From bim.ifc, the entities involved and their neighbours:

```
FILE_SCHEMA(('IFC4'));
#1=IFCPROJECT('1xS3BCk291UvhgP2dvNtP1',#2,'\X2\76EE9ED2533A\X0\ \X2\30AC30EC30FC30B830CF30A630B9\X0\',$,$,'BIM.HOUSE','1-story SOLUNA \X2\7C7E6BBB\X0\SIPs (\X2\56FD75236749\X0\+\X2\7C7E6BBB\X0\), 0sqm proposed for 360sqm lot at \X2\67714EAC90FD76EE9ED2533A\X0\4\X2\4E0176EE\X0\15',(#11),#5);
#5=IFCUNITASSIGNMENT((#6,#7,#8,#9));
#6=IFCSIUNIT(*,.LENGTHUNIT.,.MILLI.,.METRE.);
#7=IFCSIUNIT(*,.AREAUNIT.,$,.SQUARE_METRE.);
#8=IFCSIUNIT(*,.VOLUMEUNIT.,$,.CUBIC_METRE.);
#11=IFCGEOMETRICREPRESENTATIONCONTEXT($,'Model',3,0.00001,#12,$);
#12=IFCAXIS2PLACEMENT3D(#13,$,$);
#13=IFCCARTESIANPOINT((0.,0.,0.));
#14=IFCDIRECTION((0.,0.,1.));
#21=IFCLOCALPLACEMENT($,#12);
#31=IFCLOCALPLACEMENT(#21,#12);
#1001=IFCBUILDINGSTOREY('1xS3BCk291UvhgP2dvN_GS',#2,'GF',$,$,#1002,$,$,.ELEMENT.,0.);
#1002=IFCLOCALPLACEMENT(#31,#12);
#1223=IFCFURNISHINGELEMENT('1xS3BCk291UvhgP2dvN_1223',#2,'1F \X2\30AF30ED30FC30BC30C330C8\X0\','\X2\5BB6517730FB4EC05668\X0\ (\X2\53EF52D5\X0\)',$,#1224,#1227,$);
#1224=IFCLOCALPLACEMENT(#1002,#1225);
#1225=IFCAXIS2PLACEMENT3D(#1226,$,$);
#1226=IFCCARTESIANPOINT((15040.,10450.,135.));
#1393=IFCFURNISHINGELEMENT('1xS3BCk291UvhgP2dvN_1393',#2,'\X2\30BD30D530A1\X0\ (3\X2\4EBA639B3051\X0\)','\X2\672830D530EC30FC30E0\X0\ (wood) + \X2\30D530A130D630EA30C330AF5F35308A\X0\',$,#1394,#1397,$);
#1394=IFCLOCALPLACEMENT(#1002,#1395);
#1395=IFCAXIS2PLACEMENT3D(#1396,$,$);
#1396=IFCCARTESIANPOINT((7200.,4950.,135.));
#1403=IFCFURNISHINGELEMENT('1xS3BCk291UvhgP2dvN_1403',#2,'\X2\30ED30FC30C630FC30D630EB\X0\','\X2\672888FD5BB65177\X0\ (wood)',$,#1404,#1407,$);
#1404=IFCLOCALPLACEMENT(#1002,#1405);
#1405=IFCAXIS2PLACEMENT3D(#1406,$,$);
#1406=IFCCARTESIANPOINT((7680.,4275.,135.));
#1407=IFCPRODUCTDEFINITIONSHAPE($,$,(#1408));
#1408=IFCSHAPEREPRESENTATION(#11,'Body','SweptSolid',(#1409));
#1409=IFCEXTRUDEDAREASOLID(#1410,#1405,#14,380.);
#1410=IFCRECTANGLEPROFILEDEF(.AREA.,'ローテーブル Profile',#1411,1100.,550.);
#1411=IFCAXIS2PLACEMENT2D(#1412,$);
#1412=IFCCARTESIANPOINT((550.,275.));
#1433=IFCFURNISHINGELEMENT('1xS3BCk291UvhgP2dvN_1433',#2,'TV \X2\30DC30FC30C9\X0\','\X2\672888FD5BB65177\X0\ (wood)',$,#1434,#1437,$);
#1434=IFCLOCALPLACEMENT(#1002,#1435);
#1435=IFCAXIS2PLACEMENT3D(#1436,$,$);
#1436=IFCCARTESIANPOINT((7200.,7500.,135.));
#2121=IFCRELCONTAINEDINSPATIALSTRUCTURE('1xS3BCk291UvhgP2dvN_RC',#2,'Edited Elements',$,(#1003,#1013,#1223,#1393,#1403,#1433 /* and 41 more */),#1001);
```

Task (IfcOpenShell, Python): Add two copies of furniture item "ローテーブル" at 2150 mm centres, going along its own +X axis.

```python
import ifcopenshell
import ifcopenshell.api.geometry
import ifcopenshell.api.root
import ifcopenshell.util.element
import ifcopenshell.util.placement

model = ifcopenshell.open("bim.ifc")


def reuse_history(source, copy):
    """copy_class also copies each property set's owner history, people and application; keep the originals."""
    for rel in copy.IsDefinedBy:
        if rel.is_a("IfcRelDefinesByProperties") and (history := rel.RelatingPropertyDefinition.OwnerHistory):
            rel.RelatingPropertyDefinition.OwnerHistory = source.OwnerHistory
            ifcopenshell.util.element.remove_deep2(model, history)


source = model.by_guid("1xS3BCk291UvhgP2dvN_1403")
base = ifcopenshell.util.placement.get_local_placement(source.ObjectPlacement)
step = base[:3, 0] * 2150.0

for i in range(1, 3):
    copy = ifcopenshell.api.root.copy_class(model, product=source)
    copy.Representation = ifcopenshell.util.element.copy_deep(
        model, source.Representation, exclude=["IfcGeometricRepresentationContext", "IfcRepresentationMap"]
    )
    reuse_history(source, copy)
    matrix = base.copy()
    matrix[:3, 3] += i * step
    print("added at", matrix[:3, 3].round(3) + 0.0)
    ifcopenshell.api.geometry.edit_object_placement(model, product=copy, matrix=matrix, is_si=False)

model.write("bim_v2.ifc")
```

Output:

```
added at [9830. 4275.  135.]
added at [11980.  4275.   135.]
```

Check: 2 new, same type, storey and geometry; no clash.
